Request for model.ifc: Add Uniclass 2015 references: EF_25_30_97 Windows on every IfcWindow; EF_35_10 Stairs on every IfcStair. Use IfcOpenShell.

First a look at what the model holds.

```python
import ifcopenshell

model = ifcopenshell.open("model.ifc")
print(model.schema)
print("classifications:", [c.Name for c in model.by_type("IfcClassification")])
for ifc_class in ("IfcDoor", "IfcRoof", "IfcStair", "IfcWall", "IfcWindow"):
    print(ifc_class, len(model.by_type(ifc_class)))
```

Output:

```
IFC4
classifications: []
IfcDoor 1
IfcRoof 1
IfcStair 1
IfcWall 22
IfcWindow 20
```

```python
import ifcopenshell
import ifcopenshell.api.classification

model = ifcopenshell.open("model.ifc")

system = ifcopenshell.api.classification.add_classification(model, classification="Uniclass 2015")

codes = {
    "IfcWindow": ("EF_25_30_97", "Windows"),
    "IfcStair": ("EF_35_10", "Stairs"),
}
for ifc_class, (code, name) in codes.items():
    products = model.by_type(ifc_class)
    ifcopenshell.api.classification.add_reference(
        model, products=products, classification=system, identification=code, name=name
    )
    print(code, len(products))

model.write("model_updated.ifc")
```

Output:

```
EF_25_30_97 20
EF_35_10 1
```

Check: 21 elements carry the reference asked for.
